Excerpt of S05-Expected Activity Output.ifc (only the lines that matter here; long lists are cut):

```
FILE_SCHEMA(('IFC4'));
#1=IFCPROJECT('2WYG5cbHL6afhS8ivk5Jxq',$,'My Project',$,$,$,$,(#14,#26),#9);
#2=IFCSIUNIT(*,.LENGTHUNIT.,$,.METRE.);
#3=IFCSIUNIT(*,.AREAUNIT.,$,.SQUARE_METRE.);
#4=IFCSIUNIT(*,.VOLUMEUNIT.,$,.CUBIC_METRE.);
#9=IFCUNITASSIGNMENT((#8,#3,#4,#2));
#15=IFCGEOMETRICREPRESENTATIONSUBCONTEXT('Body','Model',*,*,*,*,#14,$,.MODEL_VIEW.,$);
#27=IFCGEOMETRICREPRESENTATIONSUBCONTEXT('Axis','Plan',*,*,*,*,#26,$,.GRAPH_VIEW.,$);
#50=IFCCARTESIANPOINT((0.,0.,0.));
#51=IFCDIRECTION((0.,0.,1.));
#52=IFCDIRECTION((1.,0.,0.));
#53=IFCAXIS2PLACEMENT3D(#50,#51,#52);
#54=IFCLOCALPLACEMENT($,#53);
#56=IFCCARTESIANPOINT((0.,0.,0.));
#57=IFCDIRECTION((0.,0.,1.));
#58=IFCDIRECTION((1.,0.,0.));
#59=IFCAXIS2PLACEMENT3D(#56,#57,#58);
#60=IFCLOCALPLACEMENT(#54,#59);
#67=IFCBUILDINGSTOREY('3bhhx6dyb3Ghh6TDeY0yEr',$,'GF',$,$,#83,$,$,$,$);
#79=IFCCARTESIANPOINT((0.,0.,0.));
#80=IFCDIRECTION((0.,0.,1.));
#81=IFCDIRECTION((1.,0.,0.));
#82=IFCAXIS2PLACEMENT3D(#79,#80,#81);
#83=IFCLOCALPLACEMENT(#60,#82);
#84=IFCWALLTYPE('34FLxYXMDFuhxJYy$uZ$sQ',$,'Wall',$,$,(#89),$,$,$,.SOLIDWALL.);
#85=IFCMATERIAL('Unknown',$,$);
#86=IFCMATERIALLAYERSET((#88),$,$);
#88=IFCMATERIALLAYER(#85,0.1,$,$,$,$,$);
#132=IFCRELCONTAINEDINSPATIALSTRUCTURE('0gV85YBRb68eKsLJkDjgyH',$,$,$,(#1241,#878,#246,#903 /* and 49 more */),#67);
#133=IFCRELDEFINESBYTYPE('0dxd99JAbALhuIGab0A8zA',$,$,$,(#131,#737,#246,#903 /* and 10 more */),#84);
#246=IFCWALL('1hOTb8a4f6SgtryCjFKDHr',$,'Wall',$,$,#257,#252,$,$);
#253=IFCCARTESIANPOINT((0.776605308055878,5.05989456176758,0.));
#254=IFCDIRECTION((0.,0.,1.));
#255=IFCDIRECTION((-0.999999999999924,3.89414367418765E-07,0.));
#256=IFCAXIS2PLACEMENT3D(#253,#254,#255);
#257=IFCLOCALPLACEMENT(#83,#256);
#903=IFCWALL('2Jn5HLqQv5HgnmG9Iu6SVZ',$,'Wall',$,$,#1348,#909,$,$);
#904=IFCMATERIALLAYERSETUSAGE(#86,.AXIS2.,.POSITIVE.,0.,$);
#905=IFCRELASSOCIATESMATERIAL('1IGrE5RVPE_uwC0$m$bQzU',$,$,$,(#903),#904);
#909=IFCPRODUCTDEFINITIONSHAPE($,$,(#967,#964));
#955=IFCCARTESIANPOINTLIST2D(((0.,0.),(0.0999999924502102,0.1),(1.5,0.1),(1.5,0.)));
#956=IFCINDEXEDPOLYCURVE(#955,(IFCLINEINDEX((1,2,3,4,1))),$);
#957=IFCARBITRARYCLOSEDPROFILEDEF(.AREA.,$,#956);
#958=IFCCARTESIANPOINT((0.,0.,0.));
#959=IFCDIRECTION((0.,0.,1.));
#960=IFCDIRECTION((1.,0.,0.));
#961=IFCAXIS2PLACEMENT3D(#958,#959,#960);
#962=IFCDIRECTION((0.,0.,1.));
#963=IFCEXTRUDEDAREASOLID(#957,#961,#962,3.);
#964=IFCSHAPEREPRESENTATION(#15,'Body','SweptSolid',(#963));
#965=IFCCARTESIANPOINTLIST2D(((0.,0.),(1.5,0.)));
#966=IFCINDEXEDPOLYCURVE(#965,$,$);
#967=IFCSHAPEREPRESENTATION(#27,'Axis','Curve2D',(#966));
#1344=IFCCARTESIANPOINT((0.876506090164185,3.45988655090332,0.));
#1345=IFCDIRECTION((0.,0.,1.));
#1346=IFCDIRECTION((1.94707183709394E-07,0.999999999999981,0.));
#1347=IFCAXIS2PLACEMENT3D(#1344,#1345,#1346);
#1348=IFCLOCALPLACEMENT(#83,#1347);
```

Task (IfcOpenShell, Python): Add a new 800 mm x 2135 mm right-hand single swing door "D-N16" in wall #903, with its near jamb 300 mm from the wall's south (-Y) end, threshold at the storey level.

```python
import numpy as np
import ifcopenshell
import ifcopenshell.api.feature
import ifcopenshell.api.geometry
import ifcopenshell.api.root
import ifcopenshell.api.spatial
import ifcopenshell.geom
import ifcopenshell.util.element
import ifcopenshell.util.placement
import ifcopenshell.util.representation
import ifcopenshell.util.shape
import ifcopenshell.util.unit

model = ifcopenshell.open("S05-Expected Activity Output.ifc")
unit_scale = ifcopenshell.util.unit.calculate_unit_scale(model)
settings = ifcopenshell.geom.settings()


def volume(element):
    """Net volume in cubic metres, openings subtracted."""
    shape = ifcopenshell.geom.create_shape(settings, element)
    return ifcopenshell.util.shape.get_volume(shape.geometry)


wall = model.by_guid("2Jn5HLqQv5HgnmG9Iu6SVZ")
storey = ifcopenshell.util.element.get_container(wall, ifc_class="IfcBuildingStorey")
context = ifcopenshell.util.representation.get_context(model, "Model", "Body", "MODEL_VIEW")
before = volume(wall)

width, height, from_end, sill = 0.8, 2.135, 0.3, 0.0  # metres

# The wall runs along its own X axis, and the end named is its -X end.
wall_shape = ifcopenshell.geom.create_shape(settings, wall)
x, y, z = ifcopenshell.util.shape.get_vertices(wall_shape.geometry).T
start = x.min() + from_end
face, thickness = float(y.min()), float(y.max() - y.min())
wall_matrix = ifcopenshell.util.placement.get_local_placement(wall.ObjectPlacement)
level = ifcopenshell.util.placement.get_local_placement(storey.ObjectPlacement)[2, 3]


def in_wall(x, y):
    """Placement at x, y metres in the wall's axes, at sill height."""
    matrix = wall_matrix.copy()
    matrix[:, 3] = wall_matrix @ np.array([x / unit_scale, y / unit_scale, 0.0, 1.0])
    matrix[2, 3] = level + sill / unit_scale
    return matrix


# Opening: a box that overshoots both wall faces by 50 mm.
opening = ifcopenshell.api.root.create_entity(model, ifc_class="IfcOpeningElement", predefined_type="OPENING")
box = ifcopenshell.api.geometry.add_wall_representation(
    model, context=context, length=width, height=height, thickness=thickness + 0.1
)
ifcopenshell.api.geometry.assign_representation(model, product=opening, representation=box)
ifcopenshell.api.geometry.edit_object_placement(model, product=opening, matrix=in_wall(start, face - 0.05), is_si=False)
ifcopenshell.api.feature.add_feature(model, feature=opening, element=wall)

door = ifcopenshell.api.root.create_entity(model, ifc_class="IfcDoor", name="D-N16", predefined_type="DOOR")
door.OverallWidth, door.OverallHeight = width / unit_scale, height / unit_scale
door.OperationType = "SINGLE_SWING_RIGHT"
body = ifcopenshell.api.geometry.add_door_representation(
    model,
    context=context,
    overall_width=door.OverallWidth,
    overall_height=door.OverallHeight,
    operation_type="SINGLE_SWING_RIGHT",
    lining_properties={"LiningDepth": thickness / unit_scale, "ThresholdDepth": thickness / unit_scale},
)
ifcopenshell.api.geometry.assign_representation(model, product=door, representation=body)
ifcopenshell.api.spatial.assign_container(model, products=[door], relating_structure=storey)
ifcopenshell.api.feature.add_filling(model, opening=opening, element=door)

# The lining spans the wall, so the door starts at the wall face.
ifcopenshell.api.geometry.edit_object_placement(model, product=door, matrix=in_wall(start, face), is_si=False)

after = volume(wall)

print(f"wall volume {before:.3f} -> {after:.3f} m3")

model.write("S05-Expected Activity Output-out.ifc")
```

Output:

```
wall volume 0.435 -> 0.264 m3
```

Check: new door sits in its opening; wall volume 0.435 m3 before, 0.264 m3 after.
